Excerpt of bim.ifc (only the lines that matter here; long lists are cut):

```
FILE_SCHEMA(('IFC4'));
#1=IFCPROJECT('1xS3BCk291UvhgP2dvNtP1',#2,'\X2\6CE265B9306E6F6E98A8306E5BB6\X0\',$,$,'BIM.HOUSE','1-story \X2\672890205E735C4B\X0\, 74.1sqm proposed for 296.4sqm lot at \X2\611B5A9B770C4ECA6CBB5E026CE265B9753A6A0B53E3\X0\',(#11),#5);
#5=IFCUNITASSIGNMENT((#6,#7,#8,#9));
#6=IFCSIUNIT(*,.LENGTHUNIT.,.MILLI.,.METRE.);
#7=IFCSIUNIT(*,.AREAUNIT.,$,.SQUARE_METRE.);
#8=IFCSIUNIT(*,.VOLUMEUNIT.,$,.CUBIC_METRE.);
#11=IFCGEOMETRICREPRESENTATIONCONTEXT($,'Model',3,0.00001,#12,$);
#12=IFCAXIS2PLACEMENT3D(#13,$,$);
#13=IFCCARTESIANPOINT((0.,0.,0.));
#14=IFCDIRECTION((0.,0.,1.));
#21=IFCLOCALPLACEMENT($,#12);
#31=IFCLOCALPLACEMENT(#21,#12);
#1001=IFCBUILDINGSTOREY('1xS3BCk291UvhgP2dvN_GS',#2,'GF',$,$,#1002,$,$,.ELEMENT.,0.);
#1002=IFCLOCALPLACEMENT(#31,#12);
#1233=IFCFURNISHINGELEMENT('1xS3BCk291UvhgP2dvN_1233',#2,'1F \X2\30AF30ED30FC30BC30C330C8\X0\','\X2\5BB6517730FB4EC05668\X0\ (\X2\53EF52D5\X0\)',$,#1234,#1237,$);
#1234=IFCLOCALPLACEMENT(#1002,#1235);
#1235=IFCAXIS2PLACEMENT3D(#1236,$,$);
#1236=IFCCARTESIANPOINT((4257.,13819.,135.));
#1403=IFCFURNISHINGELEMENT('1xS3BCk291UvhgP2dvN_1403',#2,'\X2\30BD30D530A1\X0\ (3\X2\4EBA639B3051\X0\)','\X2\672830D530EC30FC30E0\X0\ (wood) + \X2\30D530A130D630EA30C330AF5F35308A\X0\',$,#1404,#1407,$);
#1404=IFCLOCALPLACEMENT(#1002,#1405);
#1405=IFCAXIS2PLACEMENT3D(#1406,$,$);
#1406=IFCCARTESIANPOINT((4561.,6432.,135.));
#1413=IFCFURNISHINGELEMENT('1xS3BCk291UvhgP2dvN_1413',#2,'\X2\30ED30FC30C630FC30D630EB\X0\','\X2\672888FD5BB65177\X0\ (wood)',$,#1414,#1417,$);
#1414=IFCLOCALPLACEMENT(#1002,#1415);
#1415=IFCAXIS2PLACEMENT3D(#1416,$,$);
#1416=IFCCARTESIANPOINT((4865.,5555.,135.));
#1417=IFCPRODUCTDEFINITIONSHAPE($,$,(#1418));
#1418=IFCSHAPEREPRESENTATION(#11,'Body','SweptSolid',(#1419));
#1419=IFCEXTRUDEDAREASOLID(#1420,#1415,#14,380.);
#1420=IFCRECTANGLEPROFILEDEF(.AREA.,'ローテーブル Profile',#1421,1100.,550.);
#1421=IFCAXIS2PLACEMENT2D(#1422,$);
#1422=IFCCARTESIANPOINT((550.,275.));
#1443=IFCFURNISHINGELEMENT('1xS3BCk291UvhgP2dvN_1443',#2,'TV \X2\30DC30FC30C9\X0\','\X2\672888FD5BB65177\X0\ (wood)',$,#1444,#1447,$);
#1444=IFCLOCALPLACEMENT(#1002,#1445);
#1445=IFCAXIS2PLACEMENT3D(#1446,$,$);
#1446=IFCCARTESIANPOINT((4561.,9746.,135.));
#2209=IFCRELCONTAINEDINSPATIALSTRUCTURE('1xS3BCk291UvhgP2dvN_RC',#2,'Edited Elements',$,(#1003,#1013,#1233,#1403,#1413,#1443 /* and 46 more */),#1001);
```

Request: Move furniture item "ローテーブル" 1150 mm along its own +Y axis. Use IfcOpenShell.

```python
import ifcopenshell
import ifcopenshell.api.geometry
import ifcopenshell.util.placement

model = ifcopenshell.open("bim.ifc")

item = model.by_guid("1xS3BCk291UvhgP2dvN_1413")
matrix = ifcopenshell.util.placement.get_local_placement(item.ObjectPlacement)
matrix[:3, 3] += matrix[:3, 1] * 1150.0
ifcopenshell.api.geometry.edit_object_placement(model, product=item, matrix=matrix, is_si=False)

print(ifcopenshell.util.placement.get_local_placement(item.ObjectPlacement).round(3) + 0.0)

model.write("bim-out.ifc")
```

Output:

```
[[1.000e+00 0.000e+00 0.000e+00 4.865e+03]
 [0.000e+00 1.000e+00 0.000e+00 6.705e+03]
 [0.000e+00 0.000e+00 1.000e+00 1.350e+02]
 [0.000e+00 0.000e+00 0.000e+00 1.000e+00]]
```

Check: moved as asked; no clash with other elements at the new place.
